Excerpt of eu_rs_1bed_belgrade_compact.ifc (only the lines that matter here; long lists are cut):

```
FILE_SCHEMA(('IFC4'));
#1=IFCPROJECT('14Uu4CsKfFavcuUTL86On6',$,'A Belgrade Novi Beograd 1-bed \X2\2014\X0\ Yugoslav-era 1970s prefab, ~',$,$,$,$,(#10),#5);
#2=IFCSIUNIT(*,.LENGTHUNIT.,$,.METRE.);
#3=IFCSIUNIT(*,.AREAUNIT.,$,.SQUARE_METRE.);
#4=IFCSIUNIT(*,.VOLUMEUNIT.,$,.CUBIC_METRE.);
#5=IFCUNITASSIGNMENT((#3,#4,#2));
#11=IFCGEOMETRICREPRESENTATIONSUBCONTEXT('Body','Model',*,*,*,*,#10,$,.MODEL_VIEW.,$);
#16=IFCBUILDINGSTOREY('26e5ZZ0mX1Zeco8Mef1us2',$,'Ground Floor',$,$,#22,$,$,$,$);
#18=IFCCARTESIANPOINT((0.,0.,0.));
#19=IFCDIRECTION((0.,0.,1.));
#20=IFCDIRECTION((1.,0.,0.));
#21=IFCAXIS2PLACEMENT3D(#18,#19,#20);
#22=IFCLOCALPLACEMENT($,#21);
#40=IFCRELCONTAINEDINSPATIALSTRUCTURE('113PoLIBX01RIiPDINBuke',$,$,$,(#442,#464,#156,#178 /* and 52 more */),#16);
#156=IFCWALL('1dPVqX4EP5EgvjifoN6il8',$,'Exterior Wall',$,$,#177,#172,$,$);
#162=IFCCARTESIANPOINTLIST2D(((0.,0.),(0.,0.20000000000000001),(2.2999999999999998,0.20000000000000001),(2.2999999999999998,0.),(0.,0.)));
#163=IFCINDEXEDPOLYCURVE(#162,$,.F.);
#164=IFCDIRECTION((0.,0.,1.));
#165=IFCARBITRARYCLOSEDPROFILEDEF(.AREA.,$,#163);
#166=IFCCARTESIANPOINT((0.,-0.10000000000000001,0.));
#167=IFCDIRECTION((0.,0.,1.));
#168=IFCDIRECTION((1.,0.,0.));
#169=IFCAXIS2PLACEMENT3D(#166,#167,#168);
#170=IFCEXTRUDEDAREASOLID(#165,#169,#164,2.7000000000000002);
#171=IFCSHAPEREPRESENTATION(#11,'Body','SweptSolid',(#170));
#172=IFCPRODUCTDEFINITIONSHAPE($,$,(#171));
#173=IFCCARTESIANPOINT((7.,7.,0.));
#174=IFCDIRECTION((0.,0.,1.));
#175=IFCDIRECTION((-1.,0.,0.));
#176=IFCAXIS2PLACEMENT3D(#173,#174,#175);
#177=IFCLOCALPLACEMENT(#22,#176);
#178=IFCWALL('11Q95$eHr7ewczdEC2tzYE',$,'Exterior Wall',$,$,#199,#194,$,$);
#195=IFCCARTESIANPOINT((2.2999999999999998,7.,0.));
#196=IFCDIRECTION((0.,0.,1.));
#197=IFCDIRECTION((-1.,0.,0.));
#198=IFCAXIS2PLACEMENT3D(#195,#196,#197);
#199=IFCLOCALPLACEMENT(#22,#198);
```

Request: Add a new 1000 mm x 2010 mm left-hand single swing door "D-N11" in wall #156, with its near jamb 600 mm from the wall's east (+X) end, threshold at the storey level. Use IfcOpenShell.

```python
import numpy as np
import ifcopenshell
import ifcopenshell.api.feature
import ifcopenshell.api.geometry
import ifcopenshell.api.root
import ifcopenshell.api.spatial
import ifcopenshell.geom
import ifcopenshell.util.element
import ifcopenshell.util.placement
import ifcopenshell.util.representation
import ifcopenshell.util.shape
import ifcopenshell.util.unit

model = ifcopenshell.open("eu_rs_1bed_belgrade_compact.ifc")
unit_scale = ifcopenshell.util.unit.calculate_unit_scale(model)
settings = ifcopenshell.geom.settings()


def volume(element):
    """Net volume in cubic metres, openings subtracted."""
    shape = ifcopenshell.geom.create_shape(settings, element)
    return ifcopenshell.util.shape.get_volume(shape.geometry)


wall = model.by_id(156)
storey = ifcopenshell.util.element.get_container(wall, ifc_class="IfcBuildingStorey")
context = ifcopenshell.util.representation.get_context(model, "Model", "Body", "MODEL_VIEW")
before = volume(wall)

width, height, from_end, sill = 1, 2.01, 0.6, 0.0  # metres

# The wall runs along its own X axis, and the end named is its -X end.
wall_shape = ifcopenshell.geom.create_shape(settings, wall)
x, y, z = ifcopenshell.util.shape.get_vertices(wall_shape.geometry).T
start = x.min() + from_end
face, thickness = float(y.min()), float(y.max() - y.min())
wall_matrix = ifcopenshell.util.placement.get_local_placement(wall.ObjectPlacement)
level = ifcopenshell.util.placement.get_local_placement(storey.ObjectPlacement)[2, 3]


def in_wall(x, y):
    """Placement at x, y metres in the wall's axes, at sill height."""
    matrix = wall_matrix.copy()
    matrix[:, 3] = wall_matrix @ np.array([x / unit_scale, y / unit_scale, 0.0, 1.0])
    matrix[2, 3] = level + sill / unit_scale
    return matrix


# Opening: a box that overshoots both wall faces by 50 mm.
opening = ifcopenshell.api.root.create_entity(model, ifc_class="IfcOpeningElement", predefined_type="OPENING")
box = ifcopenshell.api.geometry.add_wall_representation(
    model, context=context, length=width, height=height, thickness=thickness + 0.1
)
ifcopenshell.api.geometry.assign_representation(model, product=opening, representation=box)
ifcopenshell.api.geometry.edit_object_placement(model, product=opening, matrix=in_wall(start, face - 0.05), is_si=False)
ifcopenshell.api.feature.add_feature(model, feature=opening, element=wall)

door = ifcopenshell.api.root.create_entity(model, ifc_class="IfcDoor", name="D-N11", predefined_type="DOOR")
door.OverallWidth, door.OverallHeight = width / unit_scale, height / unit_scale
door.OperationType = "SINGLE_SWING_LEFT"
body = ifcopenshell.api.geometry.add_door_representation(
    model,
    context=context,
    overall_width=door.OverallWidth,
    overall_height=door.OverallHeight,
    operation_type="SINGLE_SWING_LEFT",
    lining_properties={"LiningDepth": thickness / unit_scale, "ThresholdDepth": thickness / unit_scale},
)
ifcopenshell.api.geometry.assign_representation(model, product=door, representation=body)
ifcopenshell.api.spatial.assign_container(model, products=[door], relating_structure=storey)
ifcopenshell.api.feature.add_filling(model, opening=opening, element=door)

# The lining spans the wall, so the door starts at the wall face.
ifcopenshell.api.geometry.edit_object_placement(model, product=door, matrix=in_wall(start, face), is_si=False)

after = volume(wall)

print(f"wall volume {before:.3f} -> {after:.3f} m3")

model.write("eu_rs_1bed_belgrade_compact_rev.ifc")
```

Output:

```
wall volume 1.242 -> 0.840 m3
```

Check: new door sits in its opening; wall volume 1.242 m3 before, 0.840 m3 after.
